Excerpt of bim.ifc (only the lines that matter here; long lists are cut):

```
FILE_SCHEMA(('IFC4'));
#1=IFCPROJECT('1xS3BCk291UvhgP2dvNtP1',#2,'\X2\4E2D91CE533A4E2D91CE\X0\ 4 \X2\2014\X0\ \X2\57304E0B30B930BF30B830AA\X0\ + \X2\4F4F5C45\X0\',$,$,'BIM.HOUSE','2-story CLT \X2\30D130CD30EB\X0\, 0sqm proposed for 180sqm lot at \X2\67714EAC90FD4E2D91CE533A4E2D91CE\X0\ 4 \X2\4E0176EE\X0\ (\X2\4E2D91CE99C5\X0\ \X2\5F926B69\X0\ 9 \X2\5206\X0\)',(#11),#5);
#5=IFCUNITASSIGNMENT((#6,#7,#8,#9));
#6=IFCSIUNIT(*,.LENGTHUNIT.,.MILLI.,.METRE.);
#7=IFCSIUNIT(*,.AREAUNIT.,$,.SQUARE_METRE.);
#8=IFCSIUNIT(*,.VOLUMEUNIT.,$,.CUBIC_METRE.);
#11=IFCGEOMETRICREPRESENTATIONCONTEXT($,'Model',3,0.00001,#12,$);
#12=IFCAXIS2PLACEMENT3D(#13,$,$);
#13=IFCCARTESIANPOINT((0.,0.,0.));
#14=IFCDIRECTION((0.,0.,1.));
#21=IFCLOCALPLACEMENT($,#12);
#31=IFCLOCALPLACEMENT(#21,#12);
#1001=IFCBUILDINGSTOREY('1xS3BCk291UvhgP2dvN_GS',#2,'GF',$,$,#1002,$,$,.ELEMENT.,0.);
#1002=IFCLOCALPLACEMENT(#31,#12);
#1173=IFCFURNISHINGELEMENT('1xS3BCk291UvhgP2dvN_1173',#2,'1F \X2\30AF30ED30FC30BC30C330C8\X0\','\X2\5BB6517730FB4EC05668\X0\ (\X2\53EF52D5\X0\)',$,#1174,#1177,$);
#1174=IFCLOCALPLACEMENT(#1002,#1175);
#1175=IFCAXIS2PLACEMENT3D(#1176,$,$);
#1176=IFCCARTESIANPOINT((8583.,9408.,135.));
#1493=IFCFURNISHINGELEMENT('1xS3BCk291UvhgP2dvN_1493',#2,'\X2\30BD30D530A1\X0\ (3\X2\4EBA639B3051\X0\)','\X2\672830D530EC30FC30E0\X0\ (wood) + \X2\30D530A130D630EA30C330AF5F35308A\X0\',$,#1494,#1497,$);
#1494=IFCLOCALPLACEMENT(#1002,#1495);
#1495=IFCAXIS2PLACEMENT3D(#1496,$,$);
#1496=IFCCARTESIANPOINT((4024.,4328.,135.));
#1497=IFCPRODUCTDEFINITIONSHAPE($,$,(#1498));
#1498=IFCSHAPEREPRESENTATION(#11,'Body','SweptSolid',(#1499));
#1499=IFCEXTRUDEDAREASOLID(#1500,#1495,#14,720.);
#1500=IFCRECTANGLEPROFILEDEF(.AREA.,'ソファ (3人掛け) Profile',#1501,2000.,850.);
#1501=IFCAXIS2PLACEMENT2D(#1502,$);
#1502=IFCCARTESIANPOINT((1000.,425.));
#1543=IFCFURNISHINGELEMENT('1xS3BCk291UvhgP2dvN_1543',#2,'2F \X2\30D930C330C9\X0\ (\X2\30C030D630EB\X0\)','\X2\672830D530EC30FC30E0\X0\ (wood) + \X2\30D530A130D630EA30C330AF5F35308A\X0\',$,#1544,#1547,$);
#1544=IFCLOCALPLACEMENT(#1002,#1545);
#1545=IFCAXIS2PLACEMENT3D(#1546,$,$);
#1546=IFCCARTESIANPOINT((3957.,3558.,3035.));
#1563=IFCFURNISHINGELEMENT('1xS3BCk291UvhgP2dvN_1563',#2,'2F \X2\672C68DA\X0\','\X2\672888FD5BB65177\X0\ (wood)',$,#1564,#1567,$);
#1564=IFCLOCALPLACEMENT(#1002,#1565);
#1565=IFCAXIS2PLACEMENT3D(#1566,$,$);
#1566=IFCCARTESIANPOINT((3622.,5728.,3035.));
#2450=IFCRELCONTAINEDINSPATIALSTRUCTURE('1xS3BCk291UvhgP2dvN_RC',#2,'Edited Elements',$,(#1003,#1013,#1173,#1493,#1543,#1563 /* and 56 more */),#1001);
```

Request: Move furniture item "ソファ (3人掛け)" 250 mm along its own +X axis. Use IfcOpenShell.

```python
import ifcopenshell
import ifcopenshell.api.geometry
import ifcopenshell.util.placement

model = ifcopenshell.open("bim.ifc")

item = model.by_id(1493)
matrix = ifcopenshell.util.placement.get_local_placement(item.ObjectPlacement)
matrix[:3, 3] += matrix[:3, 0] * 250.0
ifcopenshell.api.geometry.edit_object_placement(model, product=item, matrix=matrix, is_si=False)

print(ifcopenshell.util.placement.get_local_placement(item.ObjectPlacement).round(3) + 0.0)

model.write("bim_updated.ifc")
```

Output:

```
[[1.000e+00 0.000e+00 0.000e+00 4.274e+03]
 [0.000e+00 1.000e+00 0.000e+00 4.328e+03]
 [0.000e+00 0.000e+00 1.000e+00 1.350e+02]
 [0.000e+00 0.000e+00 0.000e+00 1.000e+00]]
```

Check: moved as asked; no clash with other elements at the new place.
